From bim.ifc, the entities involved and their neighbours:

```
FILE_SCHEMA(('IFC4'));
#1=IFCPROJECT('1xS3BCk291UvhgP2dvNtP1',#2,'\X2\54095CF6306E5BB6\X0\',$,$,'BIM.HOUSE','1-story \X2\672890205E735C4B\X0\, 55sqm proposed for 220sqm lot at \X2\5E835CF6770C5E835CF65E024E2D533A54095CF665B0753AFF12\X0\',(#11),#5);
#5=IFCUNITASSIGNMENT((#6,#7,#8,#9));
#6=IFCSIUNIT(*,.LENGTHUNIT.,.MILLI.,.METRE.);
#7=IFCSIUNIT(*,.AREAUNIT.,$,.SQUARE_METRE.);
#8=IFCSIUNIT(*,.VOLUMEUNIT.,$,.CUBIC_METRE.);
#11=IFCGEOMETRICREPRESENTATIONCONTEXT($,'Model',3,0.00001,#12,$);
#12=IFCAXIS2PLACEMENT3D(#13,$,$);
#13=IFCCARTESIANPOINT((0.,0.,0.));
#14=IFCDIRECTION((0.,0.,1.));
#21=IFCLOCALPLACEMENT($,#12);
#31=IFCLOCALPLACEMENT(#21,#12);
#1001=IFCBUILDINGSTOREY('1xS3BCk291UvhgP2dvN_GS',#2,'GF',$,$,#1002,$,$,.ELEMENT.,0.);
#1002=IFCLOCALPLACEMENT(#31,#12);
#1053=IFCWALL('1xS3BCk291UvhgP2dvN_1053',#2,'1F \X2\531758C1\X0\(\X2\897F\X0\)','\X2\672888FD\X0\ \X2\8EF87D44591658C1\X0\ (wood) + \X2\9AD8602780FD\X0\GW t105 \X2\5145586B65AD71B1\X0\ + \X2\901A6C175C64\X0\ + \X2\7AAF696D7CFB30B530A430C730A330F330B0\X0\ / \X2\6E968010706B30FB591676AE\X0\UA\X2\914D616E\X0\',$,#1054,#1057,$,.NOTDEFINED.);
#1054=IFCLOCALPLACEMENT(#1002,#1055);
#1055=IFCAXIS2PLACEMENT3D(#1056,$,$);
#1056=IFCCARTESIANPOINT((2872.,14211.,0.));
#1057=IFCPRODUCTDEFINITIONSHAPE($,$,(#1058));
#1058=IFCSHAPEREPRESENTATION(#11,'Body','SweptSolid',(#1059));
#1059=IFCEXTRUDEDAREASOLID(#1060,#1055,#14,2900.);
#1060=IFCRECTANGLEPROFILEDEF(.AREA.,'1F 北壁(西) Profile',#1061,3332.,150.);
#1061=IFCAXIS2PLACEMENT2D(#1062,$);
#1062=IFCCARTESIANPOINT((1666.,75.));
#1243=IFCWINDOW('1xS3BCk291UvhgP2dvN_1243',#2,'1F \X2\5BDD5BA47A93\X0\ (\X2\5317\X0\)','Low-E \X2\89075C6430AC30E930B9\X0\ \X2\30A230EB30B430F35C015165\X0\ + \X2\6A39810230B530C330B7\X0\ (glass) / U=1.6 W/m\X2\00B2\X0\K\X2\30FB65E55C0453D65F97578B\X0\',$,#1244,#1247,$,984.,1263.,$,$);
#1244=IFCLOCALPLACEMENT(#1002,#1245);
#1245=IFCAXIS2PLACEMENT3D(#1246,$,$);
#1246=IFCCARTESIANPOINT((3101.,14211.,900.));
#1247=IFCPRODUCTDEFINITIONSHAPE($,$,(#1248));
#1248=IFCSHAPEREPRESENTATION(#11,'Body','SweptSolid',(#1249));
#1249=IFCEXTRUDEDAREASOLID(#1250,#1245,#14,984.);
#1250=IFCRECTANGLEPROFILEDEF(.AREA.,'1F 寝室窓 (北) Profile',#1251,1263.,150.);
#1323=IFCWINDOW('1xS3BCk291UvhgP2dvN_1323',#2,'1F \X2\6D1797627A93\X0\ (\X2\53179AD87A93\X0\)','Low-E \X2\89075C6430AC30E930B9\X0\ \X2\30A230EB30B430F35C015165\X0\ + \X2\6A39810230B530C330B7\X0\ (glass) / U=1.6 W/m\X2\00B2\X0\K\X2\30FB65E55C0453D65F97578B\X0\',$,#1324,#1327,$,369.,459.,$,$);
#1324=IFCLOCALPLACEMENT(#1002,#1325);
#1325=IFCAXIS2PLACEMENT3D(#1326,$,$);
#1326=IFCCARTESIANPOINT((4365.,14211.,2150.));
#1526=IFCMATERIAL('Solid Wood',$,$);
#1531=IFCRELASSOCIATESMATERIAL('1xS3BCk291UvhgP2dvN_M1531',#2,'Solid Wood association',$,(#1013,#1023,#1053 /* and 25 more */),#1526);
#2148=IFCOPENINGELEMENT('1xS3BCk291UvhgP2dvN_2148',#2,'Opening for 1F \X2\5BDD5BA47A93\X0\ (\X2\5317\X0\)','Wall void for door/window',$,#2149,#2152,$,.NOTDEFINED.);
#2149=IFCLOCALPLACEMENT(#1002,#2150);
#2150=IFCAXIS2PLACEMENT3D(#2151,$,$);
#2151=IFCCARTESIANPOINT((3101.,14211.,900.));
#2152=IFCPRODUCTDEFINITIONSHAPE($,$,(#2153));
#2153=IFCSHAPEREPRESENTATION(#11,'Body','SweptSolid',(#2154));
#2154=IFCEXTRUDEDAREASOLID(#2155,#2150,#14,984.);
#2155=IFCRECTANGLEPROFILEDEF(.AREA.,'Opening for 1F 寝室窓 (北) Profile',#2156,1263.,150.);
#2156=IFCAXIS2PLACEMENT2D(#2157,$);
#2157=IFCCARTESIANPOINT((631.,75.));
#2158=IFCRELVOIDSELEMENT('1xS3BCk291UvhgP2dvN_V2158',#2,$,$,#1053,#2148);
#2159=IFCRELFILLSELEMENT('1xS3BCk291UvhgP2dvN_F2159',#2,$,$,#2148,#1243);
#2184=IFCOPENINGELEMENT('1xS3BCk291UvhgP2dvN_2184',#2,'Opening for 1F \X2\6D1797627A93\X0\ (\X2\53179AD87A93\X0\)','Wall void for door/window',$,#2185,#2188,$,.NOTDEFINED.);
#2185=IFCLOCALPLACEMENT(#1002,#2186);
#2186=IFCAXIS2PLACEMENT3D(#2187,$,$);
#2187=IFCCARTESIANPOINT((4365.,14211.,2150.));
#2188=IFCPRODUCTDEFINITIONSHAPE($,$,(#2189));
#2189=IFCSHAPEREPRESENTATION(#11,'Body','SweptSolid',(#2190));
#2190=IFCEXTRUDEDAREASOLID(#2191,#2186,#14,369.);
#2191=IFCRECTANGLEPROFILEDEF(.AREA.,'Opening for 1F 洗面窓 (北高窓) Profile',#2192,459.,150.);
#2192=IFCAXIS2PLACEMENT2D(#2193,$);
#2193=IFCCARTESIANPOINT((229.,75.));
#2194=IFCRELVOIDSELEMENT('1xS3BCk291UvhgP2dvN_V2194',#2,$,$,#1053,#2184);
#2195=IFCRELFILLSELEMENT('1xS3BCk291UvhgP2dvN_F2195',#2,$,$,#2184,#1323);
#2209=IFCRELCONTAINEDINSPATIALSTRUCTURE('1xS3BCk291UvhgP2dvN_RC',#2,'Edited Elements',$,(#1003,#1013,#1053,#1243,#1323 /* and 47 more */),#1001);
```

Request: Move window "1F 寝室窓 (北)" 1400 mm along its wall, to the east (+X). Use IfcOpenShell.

```python
import ifcopenshell
import ifcopenshell.api.geometry
import ifcopenshell.util.placement
import ifcopenshell.util.unit

model = ifcopenshell.open("bim.ifc")
unit_scale = ifcopenshell.util.unit.calculate_unit_scale(model)

window = model.by_guid("1xS3BCk291UvhgP2dvN_1243")
opening = window.FillsVoids[0].RelatingOpeningElement
wall = opening.VoidsElements[0].RelatingBuildingElement

wall_matrix = ifcopenshell.util.placement.get_local_placement(wall.ObjectPlacement)
shift = wall_matrix[:3, 0] * 1.4 / unit_scale
before = ifcopenshell.util.placement.get_local_placement(window.ObjectPlacement)[:3, 3].copy()

# The window is not placed relative to its opening, so move both.
for product in (opening, window):
    matrix = ifcopenshell.util.placement.get_local_placement(product.ObjectPlacement)
    matrix[:3, 3] += shift
    ifcopenshell.api.geometry.edit_object_placement(model, product=product, matrix=matrix, is_si=False)

after = ifcopenshell.util.placement.get_local_placement(window.ObjectPlacement)[:3, 3]
print("window moved by", (after - before).round(3) + 0.0)

model.write("bim_v2.ifc")
```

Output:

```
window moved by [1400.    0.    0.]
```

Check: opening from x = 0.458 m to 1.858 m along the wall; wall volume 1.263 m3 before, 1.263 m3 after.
